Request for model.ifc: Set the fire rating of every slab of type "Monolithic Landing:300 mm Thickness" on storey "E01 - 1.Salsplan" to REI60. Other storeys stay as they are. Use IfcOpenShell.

First a look at what the model holds.

```python
import ifcopenshell
import ifcopenshell.util.element

model = ifcopenshell.open("model.ifc")
print(model.schema)
storey = next(s for s in model.by_type("IfcBuildingStorey") if s.Name == "E01 - 1.Salsplan")
slabs = [e for e in ifcopenshell.util.element.get_decomposition(storey) if e.is_a("IfcSlab")]
seen = {}
for e in slabs:
    element_type = ifcopenshell.util.element.get_type(e)
    key = (element_type.Name if element_type != e and element_type else None, ifcopenshell.util.element.get_pset(e, "Pset_SlabCommon", "FireRating"))
    seen[key] = seen.get(key, 0) + 1
for (name, value), count in sorted(seen.items(), key=str):
    print(count, "x", name, "|", value)
```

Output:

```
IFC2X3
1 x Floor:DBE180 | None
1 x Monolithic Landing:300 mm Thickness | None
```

```python
import ifcopenshell
import ifcopenshell.api.pset
import ifcopenshell.util.element

model = ifcopenshell.open("model.ifc")

storey = next(s for s in model.by_type("IfcBuildingStorey") if s.Name == "E01 - 1.Salsplan")
slabs = [e for e in ifcopenshell.util.element.get_decomposition(storey) if e.is_a("IfcSlab")]

count = 0
for e in slabs:
    element_type = ifcopenshell.util.element.get_type(e)
    if element_type in (None, e) or element_type.Name != "Monolithic Landing:300 mm Thickness":
        continue
    # add_pset returns the element's existing set when there is one.
    pset = ifcopenshell.api.pset.add_pset(model, product=e, name="Pset_SlabCommon")
    ifcopenshell.api.pset.edit_pset(model, pset=pset, properties={"FireRating": "REI60"})
    count += 1

print(count, "slabs updated")

model.write("model_v2.ifc")
```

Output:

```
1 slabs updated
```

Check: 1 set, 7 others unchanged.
